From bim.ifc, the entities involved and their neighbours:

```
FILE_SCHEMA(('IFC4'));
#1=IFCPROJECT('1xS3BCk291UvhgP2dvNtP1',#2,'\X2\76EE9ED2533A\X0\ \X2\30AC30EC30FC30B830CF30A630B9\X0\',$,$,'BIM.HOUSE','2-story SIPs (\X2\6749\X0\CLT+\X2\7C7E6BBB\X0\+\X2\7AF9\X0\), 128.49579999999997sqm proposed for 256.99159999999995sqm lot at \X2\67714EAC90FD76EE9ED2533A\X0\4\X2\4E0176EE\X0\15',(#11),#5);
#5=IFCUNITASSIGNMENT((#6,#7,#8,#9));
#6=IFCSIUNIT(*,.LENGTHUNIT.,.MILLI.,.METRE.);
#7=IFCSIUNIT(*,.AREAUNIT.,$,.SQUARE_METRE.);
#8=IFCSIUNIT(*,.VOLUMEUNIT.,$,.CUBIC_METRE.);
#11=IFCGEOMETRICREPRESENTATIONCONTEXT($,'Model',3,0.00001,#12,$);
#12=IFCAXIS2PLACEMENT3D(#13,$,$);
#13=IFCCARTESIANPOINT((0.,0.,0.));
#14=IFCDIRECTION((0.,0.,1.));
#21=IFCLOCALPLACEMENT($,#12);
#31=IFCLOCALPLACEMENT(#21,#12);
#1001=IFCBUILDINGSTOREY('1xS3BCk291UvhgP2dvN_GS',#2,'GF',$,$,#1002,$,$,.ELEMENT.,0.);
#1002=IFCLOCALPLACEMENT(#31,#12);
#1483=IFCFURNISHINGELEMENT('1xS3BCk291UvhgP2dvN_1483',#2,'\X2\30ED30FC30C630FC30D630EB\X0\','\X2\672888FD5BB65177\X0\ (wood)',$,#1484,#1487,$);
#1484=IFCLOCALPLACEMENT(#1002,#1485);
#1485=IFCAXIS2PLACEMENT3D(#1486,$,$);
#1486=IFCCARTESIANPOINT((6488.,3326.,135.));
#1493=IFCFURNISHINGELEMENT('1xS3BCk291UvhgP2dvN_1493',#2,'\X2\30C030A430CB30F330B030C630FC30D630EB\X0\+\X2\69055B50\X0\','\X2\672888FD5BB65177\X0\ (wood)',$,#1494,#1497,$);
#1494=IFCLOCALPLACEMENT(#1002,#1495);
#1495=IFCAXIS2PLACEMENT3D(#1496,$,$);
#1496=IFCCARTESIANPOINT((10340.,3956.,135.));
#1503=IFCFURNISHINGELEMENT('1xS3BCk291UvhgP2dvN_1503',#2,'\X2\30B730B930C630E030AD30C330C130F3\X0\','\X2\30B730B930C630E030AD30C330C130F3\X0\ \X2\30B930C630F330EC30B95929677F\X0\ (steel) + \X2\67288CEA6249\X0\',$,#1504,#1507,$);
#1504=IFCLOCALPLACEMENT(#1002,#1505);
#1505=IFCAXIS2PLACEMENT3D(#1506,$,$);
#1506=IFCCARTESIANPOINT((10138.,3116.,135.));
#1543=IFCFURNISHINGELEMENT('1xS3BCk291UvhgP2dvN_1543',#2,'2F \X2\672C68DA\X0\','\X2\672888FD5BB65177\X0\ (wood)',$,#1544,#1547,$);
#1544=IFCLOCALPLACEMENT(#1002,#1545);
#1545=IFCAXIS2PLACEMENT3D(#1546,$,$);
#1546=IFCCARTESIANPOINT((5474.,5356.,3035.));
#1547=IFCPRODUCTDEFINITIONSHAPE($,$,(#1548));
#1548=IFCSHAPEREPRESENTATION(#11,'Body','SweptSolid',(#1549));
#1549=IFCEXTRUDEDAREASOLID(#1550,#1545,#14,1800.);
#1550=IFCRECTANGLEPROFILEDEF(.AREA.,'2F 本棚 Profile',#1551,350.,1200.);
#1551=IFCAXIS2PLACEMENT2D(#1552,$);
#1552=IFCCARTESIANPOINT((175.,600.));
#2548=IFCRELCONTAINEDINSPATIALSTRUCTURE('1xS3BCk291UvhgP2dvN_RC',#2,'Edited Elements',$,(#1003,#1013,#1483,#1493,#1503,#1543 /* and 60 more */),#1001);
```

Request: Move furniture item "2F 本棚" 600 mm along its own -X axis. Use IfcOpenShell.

```python
import ifcopenshell
import ifcopenshell.api.geometry
import ifcopenshell.util.placement

model = ifcopenshell.open("bim.ifc")

item = model.by_guid("1xS3BCk291UvhgP2dvN_1543")
matrix = ifcopenshell.util.placement.get_local_placement(item.ObjectPlacement)
matrix[:3, 3] -= matrix[:3, 0] * 600.0
ifcopenshell.api.geometry.edit_object_placement(model, product=item, matrix=matrix, is_si=False)

print(ifcopenshell.util.placement.get_local_placement(item.ObjectPlacement).round(3) + 0.0)

model.write("bim-out.ifc")
```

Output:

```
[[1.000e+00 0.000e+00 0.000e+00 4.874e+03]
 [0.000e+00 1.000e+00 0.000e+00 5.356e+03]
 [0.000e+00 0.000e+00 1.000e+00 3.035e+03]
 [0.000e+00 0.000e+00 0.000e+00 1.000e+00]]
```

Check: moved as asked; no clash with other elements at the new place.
